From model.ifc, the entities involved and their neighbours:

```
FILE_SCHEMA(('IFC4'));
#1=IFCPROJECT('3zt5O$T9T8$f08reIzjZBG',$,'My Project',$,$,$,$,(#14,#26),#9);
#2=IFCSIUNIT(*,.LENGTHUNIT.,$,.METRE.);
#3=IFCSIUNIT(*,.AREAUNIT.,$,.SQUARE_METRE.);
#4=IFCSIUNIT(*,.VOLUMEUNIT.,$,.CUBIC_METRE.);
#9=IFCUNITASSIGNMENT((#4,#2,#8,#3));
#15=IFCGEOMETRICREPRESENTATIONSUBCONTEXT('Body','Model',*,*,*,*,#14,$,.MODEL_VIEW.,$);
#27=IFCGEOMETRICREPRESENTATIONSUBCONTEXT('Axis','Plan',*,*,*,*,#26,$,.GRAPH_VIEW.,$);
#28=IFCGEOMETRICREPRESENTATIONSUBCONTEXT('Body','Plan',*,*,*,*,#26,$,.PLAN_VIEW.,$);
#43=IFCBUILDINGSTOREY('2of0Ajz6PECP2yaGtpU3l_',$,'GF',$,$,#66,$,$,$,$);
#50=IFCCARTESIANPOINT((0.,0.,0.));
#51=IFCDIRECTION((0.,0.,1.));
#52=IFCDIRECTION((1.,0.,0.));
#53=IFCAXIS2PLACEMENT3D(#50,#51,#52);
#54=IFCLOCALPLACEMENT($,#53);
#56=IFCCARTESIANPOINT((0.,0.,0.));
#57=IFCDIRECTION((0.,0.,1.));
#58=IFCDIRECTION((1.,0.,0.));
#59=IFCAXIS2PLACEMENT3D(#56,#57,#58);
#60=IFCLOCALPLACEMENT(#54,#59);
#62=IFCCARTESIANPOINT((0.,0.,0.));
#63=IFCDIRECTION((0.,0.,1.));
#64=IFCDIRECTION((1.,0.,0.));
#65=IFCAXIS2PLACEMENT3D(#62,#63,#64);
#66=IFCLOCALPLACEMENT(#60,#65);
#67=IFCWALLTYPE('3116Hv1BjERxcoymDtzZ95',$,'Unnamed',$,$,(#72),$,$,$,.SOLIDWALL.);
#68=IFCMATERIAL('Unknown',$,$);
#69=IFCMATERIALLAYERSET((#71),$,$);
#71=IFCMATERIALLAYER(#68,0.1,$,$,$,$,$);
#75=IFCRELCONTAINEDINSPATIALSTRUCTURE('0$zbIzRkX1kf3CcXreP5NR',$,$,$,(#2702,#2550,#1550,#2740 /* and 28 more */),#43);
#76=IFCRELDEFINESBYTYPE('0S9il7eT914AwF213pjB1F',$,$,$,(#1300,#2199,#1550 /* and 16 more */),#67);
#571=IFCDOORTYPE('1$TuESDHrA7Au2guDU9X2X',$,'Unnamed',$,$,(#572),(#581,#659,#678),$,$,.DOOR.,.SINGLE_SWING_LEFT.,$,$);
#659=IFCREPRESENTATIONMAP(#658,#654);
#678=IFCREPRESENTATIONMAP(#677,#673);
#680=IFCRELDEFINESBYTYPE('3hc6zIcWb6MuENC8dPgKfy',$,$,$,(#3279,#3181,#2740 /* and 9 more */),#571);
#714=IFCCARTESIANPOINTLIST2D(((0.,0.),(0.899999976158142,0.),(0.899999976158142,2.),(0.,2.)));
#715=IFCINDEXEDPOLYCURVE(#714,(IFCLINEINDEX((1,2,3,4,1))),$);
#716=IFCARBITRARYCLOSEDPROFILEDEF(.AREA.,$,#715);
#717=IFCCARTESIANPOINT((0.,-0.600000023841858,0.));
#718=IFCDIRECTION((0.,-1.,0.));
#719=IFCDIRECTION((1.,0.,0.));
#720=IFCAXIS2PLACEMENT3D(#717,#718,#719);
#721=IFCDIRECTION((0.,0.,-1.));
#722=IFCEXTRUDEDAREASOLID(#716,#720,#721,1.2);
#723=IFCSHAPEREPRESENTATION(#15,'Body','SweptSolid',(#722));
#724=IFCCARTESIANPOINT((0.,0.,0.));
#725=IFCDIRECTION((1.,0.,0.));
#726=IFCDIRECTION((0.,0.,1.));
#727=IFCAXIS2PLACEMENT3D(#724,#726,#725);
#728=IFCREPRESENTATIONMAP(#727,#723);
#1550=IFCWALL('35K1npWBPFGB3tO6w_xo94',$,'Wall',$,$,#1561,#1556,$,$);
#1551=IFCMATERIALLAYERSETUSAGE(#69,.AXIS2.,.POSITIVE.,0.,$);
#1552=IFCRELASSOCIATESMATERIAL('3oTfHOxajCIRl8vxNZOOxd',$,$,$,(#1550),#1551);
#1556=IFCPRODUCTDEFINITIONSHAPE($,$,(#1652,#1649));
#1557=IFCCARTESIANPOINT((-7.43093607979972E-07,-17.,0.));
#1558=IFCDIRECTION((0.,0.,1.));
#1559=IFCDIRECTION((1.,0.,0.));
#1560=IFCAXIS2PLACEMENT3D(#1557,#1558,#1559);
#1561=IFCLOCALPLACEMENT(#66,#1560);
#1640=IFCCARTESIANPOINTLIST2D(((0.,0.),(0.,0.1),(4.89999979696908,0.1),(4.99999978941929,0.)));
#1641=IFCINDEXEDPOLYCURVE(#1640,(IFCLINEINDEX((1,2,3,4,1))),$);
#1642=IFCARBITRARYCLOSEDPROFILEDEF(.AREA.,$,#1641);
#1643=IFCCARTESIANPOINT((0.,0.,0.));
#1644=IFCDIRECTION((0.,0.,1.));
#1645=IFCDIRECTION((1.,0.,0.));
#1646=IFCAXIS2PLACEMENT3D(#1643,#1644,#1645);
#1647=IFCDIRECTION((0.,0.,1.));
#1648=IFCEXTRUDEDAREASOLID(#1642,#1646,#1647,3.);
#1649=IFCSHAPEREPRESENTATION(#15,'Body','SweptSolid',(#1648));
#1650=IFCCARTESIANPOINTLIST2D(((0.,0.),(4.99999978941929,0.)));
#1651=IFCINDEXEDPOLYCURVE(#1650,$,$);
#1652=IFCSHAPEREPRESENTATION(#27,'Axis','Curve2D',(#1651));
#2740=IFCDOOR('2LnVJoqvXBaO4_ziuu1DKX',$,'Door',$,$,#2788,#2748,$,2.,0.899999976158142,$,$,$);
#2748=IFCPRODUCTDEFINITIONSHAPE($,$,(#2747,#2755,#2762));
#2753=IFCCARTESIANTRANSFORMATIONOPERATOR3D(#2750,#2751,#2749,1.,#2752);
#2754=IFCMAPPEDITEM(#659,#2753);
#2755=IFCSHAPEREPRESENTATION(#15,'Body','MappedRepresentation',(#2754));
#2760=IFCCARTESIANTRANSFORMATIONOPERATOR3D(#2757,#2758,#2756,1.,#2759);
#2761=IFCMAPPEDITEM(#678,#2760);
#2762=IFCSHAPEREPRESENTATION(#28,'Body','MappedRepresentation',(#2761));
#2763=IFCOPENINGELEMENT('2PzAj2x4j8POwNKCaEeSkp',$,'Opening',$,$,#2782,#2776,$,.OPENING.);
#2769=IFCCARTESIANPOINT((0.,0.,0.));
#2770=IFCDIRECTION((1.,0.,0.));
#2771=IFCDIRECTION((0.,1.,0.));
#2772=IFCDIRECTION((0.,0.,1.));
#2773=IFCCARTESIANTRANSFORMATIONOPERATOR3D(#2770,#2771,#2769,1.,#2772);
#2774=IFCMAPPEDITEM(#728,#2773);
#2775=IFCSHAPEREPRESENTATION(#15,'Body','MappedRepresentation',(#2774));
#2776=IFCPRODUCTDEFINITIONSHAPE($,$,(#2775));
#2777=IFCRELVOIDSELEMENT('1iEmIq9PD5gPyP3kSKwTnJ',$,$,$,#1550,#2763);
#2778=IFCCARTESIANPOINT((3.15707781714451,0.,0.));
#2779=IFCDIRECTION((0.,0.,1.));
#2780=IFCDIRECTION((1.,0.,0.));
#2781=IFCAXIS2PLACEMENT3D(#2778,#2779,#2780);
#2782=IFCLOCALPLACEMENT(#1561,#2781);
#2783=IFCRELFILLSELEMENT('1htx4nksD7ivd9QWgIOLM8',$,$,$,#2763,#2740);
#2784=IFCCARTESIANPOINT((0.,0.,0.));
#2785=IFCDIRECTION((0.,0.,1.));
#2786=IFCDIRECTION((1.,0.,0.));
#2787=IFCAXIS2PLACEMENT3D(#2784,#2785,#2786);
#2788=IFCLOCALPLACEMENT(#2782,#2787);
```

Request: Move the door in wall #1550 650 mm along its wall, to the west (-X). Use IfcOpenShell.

```python
import ifcopenshell
import ifcopenshell.api.geometry
import ifcopenshell.util.placement
import ifcopenshell.util.unit

model = ifcopenshell.open("model.ifc")
unit_scale = ifcopenshell.util.unit.calculate_unit_scale(model)

door = model.by_guid("2LnVJoqvXBaO4_ziuu1DKX")
opening = door.FillsVoids[0].RelatingOpeningElement
wall = opening.VoidsElements[0].RelatingBuildingElement

wall_matrix = ifcopenshell.util.placement.get_local_placement(wall.ObjectPlacement)
shift = wall_matrix[:3, 0] * -0.65 / unit_scale
before = ifcopenshell.util.placement.get_local_placement(door.ObjectPlacement)[:3, 3].copy()

# The door is placed relative to its opening, so it follows when the opening moves.
matrix = ifcopenshell.util.placement.get_local_placement(opening.ObjectPlacement)
matrix[:3, 3] += shift
ifcopenshell.api.geometry.edit_object_placement(
    model, product=opening, matrix=matrix, is_si=False, should_transform_children=True
)

after = ifcopenshell.util.placement.get_local_placement(door.ObjectPlacement)[:3, 3]
print("door moved by", (after - before).round(3) + 0.0)

model.write("model_v2.ifc")
```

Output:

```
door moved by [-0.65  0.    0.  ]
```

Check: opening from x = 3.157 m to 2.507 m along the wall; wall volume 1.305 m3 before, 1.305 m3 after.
